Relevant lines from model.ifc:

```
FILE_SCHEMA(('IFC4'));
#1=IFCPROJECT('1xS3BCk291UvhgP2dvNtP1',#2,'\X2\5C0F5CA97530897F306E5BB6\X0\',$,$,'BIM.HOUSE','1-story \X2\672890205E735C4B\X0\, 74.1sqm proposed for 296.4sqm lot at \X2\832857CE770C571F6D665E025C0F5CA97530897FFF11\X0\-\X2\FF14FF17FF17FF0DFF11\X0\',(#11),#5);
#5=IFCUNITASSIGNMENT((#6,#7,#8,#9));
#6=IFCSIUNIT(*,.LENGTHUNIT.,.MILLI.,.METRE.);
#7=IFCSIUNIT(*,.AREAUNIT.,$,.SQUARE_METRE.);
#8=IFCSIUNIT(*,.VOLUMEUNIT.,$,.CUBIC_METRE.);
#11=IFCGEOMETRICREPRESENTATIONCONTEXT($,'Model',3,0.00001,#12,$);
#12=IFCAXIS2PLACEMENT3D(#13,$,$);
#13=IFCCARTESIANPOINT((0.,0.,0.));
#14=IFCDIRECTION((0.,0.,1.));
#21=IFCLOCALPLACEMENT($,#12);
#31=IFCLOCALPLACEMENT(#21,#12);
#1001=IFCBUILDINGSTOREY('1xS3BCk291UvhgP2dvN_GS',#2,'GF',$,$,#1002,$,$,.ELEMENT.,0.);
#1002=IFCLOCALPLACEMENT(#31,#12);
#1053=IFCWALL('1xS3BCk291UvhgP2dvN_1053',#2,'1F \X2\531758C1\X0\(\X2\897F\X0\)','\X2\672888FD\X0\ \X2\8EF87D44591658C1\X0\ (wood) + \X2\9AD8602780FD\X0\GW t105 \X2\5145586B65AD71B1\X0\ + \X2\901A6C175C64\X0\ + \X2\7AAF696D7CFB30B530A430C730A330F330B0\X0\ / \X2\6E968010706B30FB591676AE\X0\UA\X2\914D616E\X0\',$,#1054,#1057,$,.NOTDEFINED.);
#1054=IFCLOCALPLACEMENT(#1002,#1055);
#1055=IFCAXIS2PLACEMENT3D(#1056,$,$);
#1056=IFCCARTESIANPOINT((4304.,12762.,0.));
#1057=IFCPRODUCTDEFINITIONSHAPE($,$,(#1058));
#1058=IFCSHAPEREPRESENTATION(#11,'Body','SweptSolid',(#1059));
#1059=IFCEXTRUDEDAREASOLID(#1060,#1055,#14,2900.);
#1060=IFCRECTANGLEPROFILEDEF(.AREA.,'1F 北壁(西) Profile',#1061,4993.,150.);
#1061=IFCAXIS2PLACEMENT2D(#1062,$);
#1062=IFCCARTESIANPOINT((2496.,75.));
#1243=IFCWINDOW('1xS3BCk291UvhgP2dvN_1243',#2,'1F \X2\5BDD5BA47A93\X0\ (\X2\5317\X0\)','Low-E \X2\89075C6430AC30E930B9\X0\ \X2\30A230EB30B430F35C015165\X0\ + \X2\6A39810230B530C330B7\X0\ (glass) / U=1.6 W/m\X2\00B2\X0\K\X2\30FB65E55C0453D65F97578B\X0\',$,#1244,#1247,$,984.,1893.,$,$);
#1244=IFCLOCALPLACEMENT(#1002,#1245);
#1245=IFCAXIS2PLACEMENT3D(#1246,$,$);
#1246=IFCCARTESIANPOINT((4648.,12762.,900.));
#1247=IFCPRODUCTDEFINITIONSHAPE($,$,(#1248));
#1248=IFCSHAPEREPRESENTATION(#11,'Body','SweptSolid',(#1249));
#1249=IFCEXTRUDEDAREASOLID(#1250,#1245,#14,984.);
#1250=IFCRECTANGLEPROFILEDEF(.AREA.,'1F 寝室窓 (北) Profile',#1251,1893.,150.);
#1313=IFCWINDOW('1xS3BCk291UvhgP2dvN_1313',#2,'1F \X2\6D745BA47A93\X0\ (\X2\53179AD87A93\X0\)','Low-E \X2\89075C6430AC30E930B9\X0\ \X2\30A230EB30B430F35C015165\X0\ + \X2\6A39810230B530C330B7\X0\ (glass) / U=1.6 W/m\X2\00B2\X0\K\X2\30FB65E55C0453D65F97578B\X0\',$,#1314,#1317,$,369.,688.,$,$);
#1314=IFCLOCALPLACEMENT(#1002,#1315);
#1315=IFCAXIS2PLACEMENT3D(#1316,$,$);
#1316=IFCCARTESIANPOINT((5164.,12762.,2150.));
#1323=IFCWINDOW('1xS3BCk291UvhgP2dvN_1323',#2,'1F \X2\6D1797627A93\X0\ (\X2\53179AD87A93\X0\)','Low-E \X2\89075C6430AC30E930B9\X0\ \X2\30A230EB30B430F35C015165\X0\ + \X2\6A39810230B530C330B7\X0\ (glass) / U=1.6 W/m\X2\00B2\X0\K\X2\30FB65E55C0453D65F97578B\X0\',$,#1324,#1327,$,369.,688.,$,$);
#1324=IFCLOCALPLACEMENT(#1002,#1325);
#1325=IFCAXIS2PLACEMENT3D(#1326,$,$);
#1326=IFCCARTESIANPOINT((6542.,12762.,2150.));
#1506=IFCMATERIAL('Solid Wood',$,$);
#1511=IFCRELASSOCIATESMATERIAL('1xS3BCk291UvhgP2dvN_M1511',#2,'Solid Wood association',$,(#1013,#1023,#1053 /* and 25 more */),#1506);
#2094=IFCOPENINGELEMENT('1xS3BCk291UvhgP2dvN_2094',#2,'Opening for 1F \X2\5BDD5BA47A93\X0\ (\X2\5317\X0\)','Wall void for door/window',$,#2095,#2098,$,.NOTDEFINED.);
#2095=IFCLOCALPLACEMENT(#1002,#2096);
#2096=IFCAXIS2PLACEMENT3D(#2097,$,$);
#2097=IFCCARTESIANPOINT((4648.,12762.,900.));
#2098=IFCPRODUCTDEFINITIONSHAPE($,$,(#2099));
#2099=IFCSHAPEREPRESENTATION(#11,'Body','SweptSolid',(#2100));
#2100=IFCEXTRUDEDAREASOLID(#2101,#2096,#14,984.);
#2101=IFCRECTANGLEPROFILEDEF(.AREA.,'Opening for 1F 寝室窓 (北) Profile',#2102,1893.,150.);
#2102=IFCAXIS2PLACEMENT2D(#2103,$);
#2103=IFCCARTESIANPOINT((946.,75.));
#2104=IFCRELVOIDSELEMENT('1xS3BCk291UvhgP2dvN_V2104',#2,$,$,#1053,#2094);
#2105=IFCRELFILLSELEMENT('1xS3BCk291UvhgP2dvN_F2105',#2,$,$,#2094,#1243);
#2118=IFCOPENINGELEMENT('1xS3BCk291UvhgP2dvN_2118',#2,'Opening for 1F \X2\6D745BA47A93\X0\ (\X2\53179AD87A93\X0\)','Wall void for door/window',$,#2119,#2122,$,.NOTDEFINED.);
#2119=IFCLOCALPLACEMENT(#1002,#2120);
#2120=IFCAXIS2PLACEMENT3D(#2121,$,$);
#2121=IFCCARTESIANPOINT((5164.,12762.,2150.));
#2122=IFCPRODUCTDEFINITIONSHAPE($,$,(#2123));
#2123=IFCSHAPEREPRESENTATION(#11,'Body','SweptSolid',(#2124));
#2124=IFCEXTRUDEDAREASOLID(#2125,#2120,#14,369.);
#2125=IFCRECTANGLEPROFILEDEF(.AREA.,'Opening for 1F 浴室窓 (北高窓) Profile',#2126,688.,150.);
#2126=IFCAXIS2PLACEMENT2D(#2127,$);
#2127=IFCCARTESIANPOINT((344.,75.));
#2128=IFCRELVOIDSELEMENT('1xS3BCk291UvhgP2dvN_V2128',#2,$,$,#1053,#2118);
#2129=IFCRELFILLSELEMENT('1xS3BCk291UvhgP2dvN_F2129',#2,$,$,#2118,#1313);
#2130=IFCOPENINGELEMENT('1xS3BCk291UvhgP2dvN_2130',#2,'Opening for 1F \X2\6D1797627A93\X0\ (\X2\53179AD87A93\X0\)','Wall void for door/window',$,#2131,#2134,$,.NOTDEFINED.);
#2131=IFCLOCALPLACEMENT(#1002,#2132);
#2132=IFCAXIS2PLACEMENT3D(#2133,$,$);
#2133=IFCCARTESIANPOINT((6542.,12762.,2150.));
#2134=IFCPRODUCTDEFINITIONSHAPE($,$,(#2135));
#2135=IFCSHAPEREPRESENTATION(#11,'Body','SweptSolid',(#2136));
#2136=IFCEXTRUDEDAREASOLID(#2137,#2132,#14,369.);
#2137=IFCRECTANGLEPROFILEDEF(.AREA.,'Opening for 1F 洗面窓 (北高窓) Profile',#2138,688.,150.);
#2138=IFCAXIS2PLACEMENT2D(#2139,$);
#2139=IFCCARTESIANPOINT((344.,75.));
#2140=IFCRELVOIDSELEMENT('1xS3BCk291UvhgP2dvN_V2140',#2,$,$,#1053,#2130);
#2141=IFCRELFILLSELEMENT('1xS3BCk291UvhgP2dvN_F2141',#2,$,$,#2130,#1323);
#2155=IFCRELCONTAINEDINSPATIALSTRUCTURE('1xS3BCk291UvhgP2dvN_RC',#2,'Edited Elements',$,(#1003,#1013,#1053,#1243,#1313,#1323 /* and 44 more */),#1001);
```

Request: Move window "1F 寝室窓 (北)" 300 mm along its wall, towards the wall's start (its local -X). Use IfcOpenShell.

```python
import ifcopenshell
import ifcopenshell.api.geometry
import ifcopenshell.util.placement

model = ifcopenshell.open("model.ifc")

window = model.by_guid("1xS3BCk291UvhgP2dvN_1243")
opening = window.FillsVoids[0].RelatingOpeningElement
wall = opening.VoidsElements[0].RelatingBuildingElement

wall_matrix = ifcopenshell.util.placement.get_local_placement(wall.ObjectPlacement)
shift = wall_matrix[:3, 0] * -300.0
before = ifcopenshell.util.placement.get_local_placement(window.ObjectPlacement)[:3, 3].copy()

# The window is not placed relative to its opening, so move both.
for product in (opening, window):
    matrix = ifcopenshell.util.placement.get_local_placement(product.ObjectPlacement)
    matrix[:3, 3] += shift
    ifcopenshell.api.geometry.edit_object_placement(model, product=product, matrix=matrix, is_si=False)

after = ifcopenshell.util.placement.get_local_placement(window.ObjectPlacement)[:3, 3]
print("window moved by", (after - before).round(3) + 0.0)

model.write("model_rev.ifc")
```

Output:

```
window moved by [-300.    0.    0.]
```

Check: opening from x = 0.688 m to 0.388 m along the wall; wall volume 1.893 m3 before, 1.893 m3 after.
